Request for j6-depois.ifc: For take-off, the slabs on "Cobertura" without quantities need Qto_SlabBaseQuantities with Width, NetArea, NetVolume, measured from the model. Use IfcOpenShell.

First a look at what the model holds.

```python
import ifcopenshell
import ifcopenshell.util.element
import ifcopenshell.util.unit

model = ifcopenshell.open("j6-depois.ifc")
print(model.schema)
for unit_type in ("LENGTHUNIT", "AREAUNIT", "VOLUMEUNIT"):
    print(unit_type, ifcopenshell.util.unit.calculate_unit_scale(model, unit_type))
storey = next(s for s in model.by_type("IfcBuildingStorey") if s.Name == "Cobertura")
slabs = [e for e in ifcopenshell.util.element.get_decomposition(storey) if e.is_a("IfcSlab")]
for e in sorted(slabs, key=lambda e: e.id()):
    print(e.id(), e.is_a(), e.Name, list(ifcopenshell.util.element.get_psets(e, qtos_only=True)), sep=" | ")
```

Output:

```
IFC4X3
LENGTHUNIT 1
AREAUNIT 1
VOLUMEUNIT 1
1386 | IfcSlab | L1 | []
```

```python
import ifcopenshell
import ifcopenshell.api.pset
import ifcopenshell.geom
import ifcopenshell.util.element
import ifcopenshell.util.shape
import ifcopenshell.util.unit

model = ifcopenshell.open("j6-depois.ifc")
unit_scale = ifcopenshell.util.unit.calculate_unit_scale(model)
area_scale = ifcopenshell.util.unit.calculate_unit_scale(model, "AREAUNIT")
volume_scale = ifcopenshell.util.unit.calculate_unit_scale(model, "VOLUMEUNIT")
settings = ifcopenshell.geom.settings()

storey = next(s for s in model.by_type("IfcBuildingStorey") if s.Name == "Cobertura")
slabs = [e for e in ifcopenshell.util.element.get_decomposition(storey) if e.is_a("IfcSlab")]

for e in sorted(slabs, key=lambda e: e.id()):
    if ifcopenshell.util.element.get_psets(e, qtos_only=True, should_inherit=False):
        continue
    # Geometry comes back in metres, in the element's own axes.
    shape = ifcopenshell.geom.create_shape(settings, e)
    values = {
        "Width": ifcopenshell.util.shape.get_z(shape.geometry) / unit_scale,
        "NetArea": ifcopenshell.util.shape.get_footprint_area(shape.geometry) / area_scale,
        "NetVolume": ifcopenshell.util.shape.get_volume(shape.geometry) / volume_scale,
    }
    qto = ifcopenshell.api.pset.add_qto(model, product=e, name="Qto_SlabBaseQuantities")
    ifcopenshell.api.pset.edit_qto(model, qto=qto, properties=values)
    print(e.id(), {k: round(v, 3) for k, v in values.items()})

model.write("j6-depois-out.ifc")
```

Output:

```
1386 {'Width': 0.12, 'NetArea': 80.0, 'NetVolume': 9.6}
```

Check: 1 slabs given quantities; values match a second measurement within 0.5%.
